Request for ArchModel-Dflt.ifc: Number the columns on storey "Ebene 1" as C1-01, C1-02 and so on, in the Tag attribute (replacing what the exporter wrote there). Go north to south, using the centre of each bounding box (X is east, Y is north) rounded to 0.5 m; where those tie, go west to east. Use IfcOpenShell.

First a look at what the model holds.

```python
import ifcopenshell
import ifcopenshell.util.element
import ifcopenshell.util.placement

model = ifcopenshell.open("ArchModel-Dflt.ifc")
print(model.schema)
storey = next(s for s in model.by_type("IfcBuildingStorey") if s.Name == "Ebene 1")
columns = [e for e in ifcopenshell.util.element.get_decomposition(storey) if e.is_a("IfcColumn")]
for e in sorted(columns, key=lambda e: e.id()):
    origin = ifcopenshell.util.placement.get_local_placement(e.ObjectPlacement)[:3, 3]
    print(e.id(), e.Tag, e.Name, origin.round(2) + 0.0, sep=" | ")
```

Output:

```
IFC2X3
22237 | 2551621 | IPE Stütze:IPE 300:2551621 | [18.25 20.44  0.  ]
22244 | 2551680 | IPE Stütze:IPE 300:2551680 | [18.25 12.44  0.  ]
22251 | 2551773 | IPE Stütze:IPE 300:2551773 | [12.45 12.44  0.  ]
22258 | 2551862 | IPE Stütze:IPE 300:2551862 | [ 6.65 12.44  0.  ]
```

```python
import ifcopenshell
import ifcopenshell.geom
import ifcopenshell.util.element
import ifcopenshell.util.shape

model = ifcopenshell.open("ArchModel-Dflt.ifc")
settings = ifcopenshell.geom.settings()
settings.set("use-world-coords", True)


def centre(element):
    shape = ifcopenshell.geom.create_shape(settings, element)
    return ifcopenshell.util.shape.get_bbox_centroid(shape.geometry)


storey = next(s for s in model.by_type("IfcBuildingStorey") if s.Name == "Ebene 1")
columns = [e for e in ifcopenshell.util.element.get_decomposition(storey) if e.is_a("IfcColumn")]

# Insertion points can sit at a corner or the storey origin, so sort by the geometry (in metres).
centres = {e: centre(e) for e in columns}
columns.sort(key=lambda e: (-round(centres[e][1] / 0.5), centres[e][0]))

for i, e in enumerate(columns, start=1):
    number = f"C1-{i:02d}"
    e.Tag = number
    print(e.id(), number)

model.write("ArchModel-Dflt_edited.ifc")
```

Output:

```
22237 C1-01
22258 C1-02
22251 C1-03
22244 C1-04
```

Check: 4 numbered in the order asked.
